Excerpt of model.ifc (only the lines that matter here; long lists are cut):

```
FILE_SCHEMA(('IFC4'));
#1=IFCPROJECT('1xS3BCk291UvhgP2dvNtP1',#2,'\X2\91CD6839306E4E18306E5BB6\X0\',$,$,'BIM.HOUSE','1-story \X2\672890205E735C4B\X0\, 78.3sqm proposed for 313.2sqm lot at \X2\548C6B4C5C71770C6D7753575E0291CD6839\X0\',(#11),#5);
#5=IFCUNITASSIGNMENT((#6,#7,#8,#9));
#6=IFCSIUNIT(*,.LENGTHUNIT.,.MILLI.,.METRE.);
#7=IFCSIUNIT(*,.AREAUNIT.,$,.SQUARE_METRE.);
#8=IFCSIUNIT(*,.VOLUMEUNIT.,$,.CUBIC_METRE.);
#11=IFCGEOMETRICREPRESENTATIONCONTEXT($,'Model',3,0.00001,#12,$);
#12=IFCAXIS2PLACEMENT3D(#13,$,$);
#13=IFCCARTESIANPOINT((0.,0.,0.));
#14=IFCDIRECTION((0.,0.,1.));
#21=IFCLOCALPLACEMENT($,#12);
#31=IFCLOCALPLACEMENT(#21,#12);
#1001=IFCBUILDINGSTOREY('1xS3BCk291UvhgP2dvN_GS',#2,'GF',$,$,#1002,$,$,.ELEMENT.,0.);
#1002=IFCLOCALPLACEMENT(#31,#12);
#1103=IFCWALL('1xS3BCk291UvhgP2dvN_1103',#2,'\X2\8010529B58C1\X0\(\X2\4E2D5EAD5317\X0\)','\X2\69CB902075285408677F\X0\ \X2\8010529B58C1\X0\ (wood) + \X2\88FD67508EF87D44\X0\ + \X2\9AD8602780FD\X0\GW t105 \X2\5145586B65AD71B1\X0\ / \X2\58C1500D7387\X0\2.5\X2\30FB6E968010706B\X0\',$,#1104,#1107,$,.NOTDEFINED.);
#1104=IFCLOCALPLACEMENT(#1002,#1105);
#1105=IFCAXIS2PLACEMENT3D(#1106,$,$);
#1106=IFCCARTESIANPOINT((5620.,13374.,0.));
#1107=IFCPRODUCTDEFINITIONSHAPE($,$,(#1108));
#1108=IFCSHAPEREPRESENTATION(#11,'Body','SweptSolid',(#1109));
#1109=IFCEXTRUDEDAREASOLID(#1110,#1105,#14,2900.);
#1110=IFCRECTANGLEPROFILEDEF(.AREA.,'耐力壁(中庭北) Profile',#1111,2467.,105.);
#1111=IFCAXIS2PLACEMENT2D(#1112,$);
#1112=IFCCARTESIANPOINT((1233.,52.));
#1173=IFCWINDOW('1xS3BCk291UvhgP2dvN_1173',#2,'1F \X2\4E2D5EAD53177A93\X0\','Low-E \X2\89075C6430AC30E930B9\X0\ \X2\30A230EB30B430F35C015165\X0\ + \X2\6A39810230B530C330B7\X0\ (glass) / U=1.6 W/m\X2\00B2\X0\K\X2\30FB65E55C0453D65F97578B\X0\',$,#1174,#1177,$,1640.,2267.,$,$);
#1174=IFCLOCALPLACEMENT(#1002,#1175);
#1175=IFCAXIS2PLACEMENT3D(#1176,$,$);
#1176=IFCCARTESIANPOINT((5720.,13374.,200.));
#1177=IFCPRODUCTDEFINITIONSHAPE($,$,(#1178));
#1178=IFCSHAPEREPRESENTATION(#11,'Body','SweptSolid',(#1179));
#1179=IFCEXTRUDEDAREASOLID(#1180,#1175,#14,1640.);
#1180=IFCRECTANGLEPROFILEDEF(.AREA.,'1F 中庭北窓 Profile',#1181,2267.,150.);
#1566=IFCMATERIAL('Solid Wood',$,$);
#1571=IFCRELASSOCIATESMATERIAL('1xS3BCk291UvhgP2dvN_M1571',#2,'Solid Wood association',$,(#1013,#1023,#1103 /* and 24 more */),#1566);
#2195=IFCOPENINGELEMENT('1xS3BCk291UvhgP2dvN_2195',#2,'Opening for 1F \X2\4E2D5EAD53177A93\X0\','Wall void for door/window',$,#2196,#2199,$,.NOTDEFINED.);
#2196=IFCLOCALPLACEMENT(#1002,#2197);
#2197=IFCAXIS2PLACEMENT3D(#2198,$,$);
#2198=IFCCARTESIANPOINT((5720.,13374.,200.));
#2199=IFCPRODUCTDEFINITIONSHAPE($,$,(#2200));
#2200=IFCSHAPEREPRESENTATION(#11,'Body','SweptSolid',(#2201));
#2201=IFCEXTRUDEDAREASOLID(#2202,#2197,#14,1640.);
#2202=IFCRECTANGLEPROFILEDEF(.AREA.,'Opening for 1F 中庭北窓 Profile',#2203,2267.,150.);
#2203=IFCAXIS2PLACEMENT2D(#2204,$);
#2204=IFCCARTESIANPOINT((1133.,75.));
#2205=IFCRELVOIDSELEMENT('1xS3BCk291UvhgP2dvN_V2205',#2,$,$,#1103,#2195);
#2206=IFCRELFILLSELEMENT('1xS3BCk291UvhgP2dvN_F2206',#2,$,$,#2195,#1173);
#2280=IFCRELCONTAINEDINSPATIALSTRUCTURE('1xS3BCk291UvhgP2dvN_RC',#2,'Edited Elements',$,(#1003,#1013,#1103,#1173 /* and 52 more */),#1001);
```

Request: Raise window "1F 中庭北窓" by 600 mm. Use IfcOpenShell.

```python
import numpy as np
import ifcopenshell
import ifcopenshell.api.geometry
import ifcopenshell.util.placement
import ifcopenshell.util.unit

model = ifcopenshell.open("model.ifc")
unit_scale = ifcopenshell.util.unit.calculate_unit_scale(model)

window = model.by_id(1173)
opening = window.FillsVoids[0].RelatingOpeningElement
dz = 600.0

shift = np.array([0.0, 0.0, dz])
# The window is not placed relative to its opening, so move both.
for product in (opening, window):
    matrix = ifcopenshell.util.placement.get_local_placement(product.ObjectPlacement)
    matrix[:3, 3] += shift
    ifcopenshell.api.geometry.edit_object_placement(model, product=product, matrix=matrix, is_si=False)

print(f"moved by {dz * unit_scale:+.3f} m")

model.write("model_edited.ifc")
```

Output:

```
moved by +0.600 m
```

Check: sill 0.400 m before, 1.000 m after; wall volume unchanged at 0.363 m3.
